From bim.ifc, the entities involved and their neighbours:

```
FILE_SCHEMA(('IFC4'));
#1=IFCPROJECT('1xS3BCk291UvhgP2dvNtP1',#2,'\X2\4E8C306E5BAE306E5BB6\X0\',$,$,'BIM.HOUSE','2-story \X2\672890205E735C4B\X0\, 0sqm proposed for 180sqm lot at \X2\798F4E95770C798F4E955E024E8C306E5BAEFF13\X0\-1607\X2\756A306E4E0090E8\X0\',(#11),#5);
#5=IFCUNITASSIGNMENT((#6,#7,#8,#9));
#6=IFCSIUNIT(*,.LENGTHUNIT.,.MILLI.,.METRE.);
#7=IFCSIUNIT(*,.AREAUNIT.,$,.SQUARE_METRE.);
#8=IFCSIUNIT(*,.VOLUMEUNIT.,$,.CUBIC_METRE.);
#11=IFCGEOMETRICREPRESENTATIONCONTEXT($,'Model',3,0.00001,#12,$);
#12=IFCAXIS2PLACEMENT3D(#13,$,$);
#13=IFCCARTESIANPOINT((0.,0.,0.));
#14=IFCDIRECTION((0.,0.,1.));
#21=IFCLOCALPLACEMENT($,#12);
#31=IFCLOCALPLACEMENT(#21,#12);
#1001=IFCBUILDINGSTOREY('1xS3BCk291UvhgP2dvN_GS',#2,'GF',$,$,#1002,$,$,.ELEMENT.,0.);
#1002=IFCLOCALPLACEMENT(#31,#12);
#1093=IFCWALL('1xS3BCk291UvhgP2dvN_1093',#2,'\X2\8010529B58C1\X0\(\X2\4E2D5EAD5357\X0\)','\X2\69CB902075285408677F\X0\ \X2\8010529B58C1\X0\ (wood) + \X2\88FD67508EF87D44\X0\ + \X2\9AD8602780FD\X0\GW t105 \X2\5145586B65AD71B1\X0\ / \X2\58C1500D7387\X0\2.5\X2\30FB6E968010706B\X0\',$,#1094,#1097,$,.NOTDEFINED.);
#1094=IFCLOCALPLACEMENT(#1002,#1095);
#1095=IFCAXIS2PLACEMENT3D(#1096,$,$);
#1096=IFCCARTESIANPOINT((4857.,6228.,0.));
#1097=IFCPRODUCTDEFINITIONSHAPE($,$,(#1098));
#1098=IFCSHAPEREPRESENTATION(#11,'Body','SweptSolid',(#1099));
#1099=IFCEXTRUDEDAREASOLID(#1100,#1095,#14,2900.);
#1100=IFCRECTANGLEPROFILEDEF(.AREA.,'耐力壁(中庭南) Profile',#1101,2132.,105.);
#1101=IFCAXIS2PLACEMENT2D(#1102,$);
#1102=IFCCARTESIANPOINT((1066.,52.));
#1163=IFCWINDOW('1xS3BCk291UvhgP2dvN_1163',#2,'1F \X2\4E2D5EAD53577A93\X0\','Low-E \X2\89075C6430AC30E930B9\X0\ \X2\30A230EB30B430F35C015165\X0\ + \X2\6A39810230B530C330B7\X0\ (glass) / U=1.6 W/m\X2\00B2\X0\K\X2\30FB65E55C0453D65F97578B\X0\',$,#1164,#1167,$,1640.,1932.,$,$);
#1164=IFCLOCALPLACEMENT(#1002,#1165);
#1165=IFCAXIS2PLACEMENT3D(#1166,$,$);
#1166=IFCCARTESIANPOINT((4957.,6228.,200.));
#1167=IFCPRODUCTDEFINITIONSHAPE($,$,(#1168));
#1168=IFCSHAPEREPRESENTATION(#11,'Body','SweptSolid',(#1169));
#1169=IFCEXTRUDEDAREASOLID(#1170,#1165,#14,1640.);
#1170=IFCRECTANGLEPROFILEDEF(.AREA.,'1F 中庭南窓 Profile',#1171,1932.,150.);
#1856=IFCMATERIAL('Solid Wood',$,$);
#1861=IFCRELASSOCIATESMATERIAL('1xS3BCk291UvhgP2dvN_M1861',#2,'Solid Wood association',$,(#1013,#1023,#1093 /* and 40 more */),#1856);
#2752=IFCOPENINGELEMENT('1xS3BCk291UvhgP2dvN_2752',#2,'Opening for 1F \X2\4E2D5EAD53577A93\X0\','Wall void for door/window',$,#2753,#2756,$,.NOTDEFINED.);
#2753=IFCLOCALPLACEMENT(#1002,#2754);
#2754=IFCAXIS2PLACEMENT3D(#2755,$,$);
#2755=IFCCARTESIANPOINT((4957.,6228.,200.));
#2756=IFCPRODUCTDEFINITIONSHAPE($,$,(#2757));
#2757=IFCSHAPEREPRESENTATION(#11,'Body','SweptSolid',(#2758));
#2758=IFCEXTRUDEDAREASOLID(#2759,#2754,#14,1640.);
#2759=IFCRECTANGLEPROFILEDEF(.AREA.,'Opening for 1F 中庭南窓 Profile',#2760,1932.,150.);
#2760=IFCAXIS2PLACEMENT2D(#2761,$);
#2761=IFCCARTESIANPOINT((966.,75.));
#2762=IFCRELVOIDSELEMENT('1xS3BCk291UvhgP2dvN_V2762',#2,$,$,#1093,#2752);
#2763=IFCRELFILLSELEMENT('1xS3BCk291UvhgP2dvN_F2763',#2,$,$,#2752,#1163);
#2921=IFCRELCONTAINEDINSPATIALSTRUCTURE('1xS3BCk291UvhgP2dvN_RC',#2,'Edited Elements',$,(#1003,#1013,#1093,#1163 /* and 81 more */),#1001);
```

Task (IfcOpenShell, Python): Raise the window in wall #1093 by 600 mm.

```python
import numpy as np
import ifcopenshell
import ifcopenshell.api.geometry
import ifcopenshell.util.placement
import ifcopenshell.util.unit

model = ifcopenshell.open("bim.ifc")
unit_scale = ifcopenshell.util.unit.calculate_unit_scale(model)

window = model.by_id(1163)
opening = window.FillsVoids[0].RelatingOpeningElement
dz = 0.6 / unit_scale

shift = np.array([0.0, 0.0, dz])
# The window is not placed relative to its opening, so move both.
for product in (opening, window):
    matrix = ifcopenshell.util.placement.get_local_placement(product.ObjectPlacement)
    matrix[:3, 3] += shift
    ifcopenshell.api.geometry.edit_object_placement(model, product=product, matrix=matrix, is_si=False)

print(f"moved by {dz * unit_scale:+.3f} m")

model.write("bim_v2.ifc")
```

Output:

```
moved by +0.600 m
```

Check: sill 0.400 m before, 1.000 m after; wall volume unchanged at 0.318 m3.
